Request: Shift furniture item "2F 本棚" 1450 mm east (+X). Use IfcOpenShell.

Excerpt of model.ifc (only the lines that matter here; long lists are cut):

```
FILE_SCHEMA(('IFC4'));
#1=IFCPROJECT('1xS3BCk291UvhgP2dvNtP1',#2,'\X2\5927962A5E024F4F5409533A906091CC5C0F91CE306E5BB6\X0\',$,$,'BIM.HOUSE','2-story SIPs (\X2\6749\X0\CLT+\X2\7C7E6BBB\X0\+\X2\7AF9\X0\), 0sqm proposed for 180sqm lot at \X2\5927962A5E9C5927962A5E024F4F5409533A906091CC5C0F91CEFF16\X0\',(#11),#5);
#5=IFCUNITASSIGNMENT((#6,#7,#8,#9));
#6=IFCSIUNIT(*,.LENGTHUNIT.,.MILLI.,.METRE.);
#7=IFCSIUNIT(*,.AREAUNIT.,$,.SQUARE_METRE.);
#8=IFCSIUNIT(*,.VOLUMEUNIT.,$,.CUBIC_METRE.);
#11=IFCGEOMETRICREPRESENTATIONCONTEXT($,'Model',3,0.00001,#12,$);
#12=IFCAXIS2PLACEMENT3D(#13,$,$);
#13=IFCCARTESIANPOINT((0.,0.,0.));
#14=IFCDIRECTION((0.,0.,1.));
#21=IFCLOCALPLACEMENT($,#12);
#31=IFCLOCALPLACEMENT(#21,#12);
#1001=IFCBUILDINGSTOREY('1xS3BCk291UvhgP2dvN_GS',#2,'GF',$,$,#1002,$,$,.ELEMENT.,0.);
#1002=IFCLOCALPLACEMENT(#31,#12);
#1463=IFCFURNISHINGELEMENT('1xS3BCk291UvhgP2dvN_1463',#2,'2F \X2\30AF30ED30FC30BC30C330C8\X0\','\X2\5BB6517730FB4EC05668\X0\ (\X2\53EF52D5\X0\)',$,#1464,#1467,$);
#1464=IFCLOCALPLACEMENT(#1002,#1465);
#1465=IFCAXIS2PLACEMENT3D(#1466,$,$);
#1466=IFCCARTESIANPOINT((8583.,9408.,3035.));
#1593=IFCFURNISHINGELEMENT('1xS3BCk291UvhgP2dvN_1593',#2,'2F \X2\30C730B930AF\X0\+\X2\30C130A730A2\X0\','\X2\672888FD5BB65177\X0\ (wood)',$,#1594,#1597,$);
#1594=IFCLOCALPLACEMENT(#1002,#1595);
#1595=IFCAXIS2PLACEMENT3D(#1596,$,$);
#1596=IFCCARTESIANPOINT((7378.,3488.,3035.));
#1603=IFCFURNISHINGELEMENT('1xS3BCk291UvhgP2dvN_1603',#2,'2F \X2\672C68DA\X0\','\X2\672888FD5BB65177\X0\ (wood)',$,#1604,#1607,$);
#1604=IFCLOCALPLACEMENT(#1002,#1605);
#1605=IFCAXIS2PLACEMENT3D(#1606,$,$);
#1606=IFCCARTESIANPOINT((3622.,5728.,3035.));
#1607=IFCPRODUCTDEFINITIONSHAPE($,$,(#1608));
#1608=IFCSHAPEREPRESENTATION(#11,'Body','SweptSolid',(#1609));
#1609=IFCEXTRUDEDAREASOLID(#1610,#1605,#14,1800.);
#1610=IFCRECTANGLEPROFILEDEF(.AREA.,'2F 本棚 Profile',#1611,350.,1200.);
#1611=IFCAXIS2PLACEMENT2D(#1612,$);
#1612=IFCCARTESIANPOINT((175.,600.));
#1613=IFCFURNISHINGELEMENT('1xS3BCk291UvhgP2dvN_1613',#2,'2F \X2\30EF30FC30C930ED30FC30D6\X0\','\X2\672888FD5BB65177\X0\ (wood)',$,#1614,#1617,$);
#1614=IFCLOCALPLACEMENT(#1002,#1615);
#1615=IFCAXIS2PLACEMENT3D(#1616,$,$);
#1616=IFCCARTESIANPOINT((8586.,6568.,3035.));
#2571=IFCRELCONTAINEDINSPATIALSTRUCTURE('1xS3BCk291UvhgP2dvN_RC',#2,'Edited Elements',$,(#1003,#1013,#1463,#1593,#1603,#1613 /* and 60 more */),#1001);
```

```python
import ifcopenshell
import ifcopenshell.api.geometry
import ifcopenshell.util.placement
import ifcopenshell.util.unit

model = ifcopenshell.open("model.ifc")
unit_scale = ifcopenshell.util.unit.calculate_unit_scale(model)

item = model.by_guid("1xS3BCk291UvhgP2dvN_1603")
matrix = ifcopenshell.util.placement.get_local_placement(item.ObjectPlacement)
matrix[0, 3] += 1.45 / unit_scale
ifcopenshell.api.geometry.edit_object_placement(model, product=item, matrix=matrix, is_si=False)

print(ifcopenshell.util.placement.get_local_placement(item.ObjectPlacement).round(3) + 0.0)

model.write("model_updated.ifc")
```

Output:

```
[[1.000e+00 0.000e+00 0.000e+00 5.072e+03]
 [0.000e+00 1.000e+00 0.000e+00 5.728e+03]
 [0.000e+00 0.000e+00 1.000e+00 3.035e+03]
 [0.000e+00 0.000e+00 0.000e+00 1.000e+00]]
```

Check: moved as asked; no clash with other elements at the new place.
